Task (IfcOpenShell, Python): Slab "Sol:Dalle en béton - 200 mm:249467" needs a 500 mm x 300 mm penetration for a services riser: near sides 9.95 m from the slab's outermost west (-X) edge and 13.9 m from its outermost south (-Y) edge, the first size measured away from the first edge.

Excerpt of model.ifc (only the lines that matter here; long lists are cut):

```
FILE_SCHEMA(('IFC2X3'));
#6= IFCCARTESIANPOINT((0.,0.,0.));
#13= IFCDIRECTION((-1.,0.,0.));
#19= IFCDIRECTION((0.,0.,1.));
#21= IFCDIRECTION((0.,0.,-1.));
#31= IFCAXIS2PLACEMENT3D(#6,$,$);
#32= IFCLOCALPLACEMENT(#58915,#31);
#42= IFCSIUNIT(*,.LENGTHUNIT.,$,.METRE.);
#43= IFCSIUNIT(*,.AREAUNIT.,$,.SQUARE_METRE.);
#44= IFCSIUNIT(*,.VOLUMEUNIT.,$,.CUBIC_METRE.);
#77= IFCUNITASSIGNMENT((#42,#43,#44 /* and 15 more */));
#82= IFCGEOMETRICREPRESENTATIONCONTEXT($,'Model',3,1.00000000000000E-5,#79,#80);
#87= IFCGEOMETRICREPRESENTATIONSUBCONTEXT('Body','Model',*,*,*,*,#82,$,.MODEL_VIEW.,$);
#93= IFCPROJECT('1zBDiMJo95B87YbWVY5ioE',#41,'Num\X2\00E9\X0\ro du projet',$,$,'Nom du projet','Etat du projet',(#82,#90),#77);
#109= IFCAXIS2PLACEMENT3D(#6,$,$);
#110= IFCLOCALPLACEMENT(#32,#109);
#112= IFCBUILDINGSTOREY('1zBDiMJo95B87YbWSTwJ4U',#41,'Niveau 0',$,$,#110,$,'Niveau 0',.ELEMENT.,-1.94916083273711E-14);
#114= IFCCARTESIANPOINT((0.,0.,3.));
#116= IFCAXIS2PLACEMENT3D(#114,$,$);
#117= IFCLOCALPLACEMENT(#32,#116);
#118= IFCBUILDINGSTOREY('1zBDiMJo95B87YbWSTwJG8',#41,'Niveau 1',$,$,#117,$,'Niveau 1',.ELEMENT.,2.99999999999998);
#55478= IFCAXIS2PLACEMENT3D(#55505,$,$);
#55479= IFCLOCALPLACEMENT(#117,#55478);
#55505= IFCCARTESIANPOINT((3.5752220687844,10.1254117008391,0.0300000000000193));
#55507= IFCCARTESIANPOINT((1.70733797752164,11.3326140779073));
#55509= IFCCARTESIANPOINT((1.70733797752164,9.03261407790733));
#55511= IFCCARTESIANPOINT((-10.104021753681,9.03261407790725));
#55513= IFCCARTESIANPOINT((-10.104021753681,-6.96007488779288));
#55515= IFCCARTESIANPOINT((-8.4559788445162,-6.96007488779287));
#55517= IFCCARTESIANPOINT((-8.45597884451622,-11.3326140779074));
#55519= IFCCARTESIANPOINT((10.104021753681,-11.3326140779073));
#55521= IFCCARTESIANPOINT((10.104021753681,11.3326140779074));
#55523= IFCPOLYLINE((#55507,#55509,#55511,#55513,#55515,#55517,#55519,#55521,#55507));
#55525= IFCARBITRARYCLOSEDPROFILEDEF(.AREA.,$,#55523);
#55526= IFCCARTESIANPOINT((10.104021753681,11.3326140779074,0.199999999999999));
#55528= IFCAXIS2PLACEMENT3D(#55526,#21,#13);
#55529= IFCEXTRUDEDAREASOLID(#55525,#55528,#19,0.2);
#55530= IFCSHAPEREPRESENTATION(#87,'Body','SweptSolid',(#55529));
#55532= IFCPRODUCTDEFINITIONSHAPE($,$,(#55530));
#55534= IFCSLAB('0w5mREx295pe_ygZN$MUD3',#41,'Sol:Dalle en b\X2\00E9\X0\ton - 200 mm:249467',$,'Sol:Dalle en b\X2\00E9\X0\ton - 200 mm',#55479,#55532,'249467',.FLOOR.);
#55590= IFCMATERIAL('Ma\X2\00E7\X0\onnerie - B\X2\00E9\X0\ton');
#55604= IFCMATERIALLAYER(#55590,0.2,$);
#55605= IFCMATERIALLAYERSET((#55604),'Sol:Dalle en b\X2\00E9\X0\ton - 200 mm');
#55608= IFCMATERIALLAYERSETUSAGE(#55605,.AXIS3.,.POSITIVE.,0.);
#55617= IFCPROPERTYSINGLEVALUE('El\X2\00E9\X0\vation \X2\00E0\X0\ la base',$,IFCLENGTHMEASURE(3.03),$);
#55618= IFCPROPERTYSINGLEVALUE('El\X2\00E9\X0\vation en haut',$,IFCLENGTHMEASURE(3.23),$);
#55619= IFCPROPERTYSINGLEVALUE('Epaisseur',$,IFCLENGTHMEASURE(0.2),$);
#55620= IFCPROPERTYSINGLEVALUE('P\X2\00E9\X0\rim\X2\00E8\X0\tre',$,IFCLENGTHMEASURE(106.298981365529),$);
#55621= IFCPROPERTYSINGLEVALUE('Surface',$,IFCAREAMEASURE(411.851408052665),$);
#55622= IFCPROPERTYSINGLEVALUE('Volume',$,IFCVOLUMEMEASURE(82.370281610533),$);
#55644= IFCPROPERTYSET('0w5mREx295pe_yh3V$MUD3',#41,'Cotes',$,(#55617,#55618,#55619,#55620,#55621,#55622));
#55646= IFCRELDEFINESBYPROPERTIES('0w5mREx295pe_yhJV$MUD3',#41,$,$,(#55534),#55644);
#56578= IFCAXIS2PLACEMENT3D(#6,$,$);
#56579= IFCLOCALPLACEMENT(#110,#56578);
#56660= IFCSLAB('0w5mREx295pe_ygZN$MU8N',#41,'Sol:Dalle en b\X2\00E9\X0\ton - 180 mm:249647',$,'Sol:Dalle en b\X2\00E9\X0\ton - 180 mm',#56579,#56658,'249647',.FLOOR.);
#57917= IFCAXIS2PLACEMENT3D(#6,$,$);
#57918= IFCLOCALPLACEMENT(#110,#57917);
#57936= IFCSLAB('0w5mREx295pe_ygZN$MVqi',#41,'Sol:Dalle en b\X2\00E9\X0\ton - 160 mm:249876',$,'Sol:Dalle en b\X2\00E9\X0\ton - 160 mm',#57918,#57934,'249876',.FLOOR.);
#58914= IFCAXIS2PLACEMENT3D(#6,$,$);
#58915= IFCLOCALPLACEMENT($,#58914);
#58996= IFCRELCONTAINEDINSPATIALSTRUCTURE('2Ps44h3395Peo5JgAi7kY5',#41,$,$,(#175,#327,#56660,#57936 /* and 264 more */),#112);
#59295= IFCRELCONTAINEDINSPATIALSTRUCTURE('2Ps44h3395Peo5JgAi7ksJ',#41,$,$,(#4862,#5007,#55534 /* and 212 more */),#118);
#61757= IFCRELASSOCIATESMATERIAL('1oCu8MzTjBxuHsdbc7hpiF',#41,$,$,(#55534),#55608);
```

```python
import numpy as np
import ifcopenshell
import ifcopenshell.api.feature
import ifcopenshell.api.geometry
import ifcopenshell.api.pset
import ifcopenshell.api.root
import ifcopenshell.geom
import ifcopenshell.util.element
import ifcopenshell.util.placement
import ifcopenshell.util.representation
import ifcopenshell.util.shape
import ifcopenshell.util.unit

model = ifcopenshell.open("model.ifc")
unit_scale = ifcopenshell.util.unit.calculate_unit_scale(model)
area_scale = ifcopenshell.util.unit.calculate_unit_scale(model, "AREAUNIT")
volume_scale = ifcopenshell.util.unit.calculate_unit_scale(model, "VOLUMEUNIT")
settings = ifcopenshell.geom.settings()


def volume(element):
    """Net volume in cubic metres, openings subtracted."""
    shape = ifcopenshell.geom.create_shape(settings, element)
    return ifcopenshell.util.shape.get_volume(shape.geometry)


slab = model.by_guid("0w5mREx295pe_ygZN$MUD3")
before = volume(slab)

# Extent in the slab's own axes, in metres. The edges named are its -X and -Y sides.
slab_shape = ifcopenshell.geom.create_shape(settings, slab)
vertices = ifcopenshell.util.shape.get_vertices(slab_shape.geometry)
x_min, y_min, bottom = vertices.min(axis=0)
top = vertices[:, 2].max()

opening = ifcopenshell.api.root.create_entity(model, ifc_class="IfcOpeningElement", name="Services riser opening")
context = ifcopenshell.util.representation.get_context(model, "Model", "Body", "MODEL_VIEW")
width, depth = 0.5, 0.3
outline = [(0.0, 0.0), (width, 0.0), (width, depth), (0.0, depth), (0.0, 0.0)]
# Overshoot both faces by 50 mm so the cut is clean.
shape = ifcopenshell.api.geometry.add_slab_representation(
    model, context=context, depth=top - bottom + 0.1, polyline=outline
)
ifcopenshell.api.geometry.assign_representation(model, product=opening, representation=shape)

matrix = ifcopenshell.util.placement.get_local_placement(slab.ObjectPlacement)
matrix[:, 3] = matrix @ np.append(np.array([x_min + 9.95, y_min + 13.9, bottom - 0.05]) / unit_scale, 1.0)
ifcopenshell.api.geometry.edit_object_placement(model, product=opening, matrix=matrix, is_si=False)
ifcopenshell.api.feature.add_feature(model, feature=opening, element=slab)

after = volume(slab)

# Update the slab's stored quantities.
pset = model.by_id(ifcopenshell.util.element.get_pset(slab, "Cotes", should_inherit=False)["id"])
ifcopenshell.api.pset.edit_pset(model, pset=pset, properties={
    "Surface": model.create_entity("IfcAreaMeasure", after / (top - bottom) / area_scale),
    "Volume": model.create_entity("IfcVolumeMeasure", after / volume_scale),
})

print(f"slab volume {before:.3f} -> {after:.3f} m3")

model.write("model-out.ifc")
```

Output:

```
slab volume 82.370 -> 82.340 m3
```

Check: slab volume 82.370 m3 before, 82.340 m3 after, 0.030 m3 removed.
